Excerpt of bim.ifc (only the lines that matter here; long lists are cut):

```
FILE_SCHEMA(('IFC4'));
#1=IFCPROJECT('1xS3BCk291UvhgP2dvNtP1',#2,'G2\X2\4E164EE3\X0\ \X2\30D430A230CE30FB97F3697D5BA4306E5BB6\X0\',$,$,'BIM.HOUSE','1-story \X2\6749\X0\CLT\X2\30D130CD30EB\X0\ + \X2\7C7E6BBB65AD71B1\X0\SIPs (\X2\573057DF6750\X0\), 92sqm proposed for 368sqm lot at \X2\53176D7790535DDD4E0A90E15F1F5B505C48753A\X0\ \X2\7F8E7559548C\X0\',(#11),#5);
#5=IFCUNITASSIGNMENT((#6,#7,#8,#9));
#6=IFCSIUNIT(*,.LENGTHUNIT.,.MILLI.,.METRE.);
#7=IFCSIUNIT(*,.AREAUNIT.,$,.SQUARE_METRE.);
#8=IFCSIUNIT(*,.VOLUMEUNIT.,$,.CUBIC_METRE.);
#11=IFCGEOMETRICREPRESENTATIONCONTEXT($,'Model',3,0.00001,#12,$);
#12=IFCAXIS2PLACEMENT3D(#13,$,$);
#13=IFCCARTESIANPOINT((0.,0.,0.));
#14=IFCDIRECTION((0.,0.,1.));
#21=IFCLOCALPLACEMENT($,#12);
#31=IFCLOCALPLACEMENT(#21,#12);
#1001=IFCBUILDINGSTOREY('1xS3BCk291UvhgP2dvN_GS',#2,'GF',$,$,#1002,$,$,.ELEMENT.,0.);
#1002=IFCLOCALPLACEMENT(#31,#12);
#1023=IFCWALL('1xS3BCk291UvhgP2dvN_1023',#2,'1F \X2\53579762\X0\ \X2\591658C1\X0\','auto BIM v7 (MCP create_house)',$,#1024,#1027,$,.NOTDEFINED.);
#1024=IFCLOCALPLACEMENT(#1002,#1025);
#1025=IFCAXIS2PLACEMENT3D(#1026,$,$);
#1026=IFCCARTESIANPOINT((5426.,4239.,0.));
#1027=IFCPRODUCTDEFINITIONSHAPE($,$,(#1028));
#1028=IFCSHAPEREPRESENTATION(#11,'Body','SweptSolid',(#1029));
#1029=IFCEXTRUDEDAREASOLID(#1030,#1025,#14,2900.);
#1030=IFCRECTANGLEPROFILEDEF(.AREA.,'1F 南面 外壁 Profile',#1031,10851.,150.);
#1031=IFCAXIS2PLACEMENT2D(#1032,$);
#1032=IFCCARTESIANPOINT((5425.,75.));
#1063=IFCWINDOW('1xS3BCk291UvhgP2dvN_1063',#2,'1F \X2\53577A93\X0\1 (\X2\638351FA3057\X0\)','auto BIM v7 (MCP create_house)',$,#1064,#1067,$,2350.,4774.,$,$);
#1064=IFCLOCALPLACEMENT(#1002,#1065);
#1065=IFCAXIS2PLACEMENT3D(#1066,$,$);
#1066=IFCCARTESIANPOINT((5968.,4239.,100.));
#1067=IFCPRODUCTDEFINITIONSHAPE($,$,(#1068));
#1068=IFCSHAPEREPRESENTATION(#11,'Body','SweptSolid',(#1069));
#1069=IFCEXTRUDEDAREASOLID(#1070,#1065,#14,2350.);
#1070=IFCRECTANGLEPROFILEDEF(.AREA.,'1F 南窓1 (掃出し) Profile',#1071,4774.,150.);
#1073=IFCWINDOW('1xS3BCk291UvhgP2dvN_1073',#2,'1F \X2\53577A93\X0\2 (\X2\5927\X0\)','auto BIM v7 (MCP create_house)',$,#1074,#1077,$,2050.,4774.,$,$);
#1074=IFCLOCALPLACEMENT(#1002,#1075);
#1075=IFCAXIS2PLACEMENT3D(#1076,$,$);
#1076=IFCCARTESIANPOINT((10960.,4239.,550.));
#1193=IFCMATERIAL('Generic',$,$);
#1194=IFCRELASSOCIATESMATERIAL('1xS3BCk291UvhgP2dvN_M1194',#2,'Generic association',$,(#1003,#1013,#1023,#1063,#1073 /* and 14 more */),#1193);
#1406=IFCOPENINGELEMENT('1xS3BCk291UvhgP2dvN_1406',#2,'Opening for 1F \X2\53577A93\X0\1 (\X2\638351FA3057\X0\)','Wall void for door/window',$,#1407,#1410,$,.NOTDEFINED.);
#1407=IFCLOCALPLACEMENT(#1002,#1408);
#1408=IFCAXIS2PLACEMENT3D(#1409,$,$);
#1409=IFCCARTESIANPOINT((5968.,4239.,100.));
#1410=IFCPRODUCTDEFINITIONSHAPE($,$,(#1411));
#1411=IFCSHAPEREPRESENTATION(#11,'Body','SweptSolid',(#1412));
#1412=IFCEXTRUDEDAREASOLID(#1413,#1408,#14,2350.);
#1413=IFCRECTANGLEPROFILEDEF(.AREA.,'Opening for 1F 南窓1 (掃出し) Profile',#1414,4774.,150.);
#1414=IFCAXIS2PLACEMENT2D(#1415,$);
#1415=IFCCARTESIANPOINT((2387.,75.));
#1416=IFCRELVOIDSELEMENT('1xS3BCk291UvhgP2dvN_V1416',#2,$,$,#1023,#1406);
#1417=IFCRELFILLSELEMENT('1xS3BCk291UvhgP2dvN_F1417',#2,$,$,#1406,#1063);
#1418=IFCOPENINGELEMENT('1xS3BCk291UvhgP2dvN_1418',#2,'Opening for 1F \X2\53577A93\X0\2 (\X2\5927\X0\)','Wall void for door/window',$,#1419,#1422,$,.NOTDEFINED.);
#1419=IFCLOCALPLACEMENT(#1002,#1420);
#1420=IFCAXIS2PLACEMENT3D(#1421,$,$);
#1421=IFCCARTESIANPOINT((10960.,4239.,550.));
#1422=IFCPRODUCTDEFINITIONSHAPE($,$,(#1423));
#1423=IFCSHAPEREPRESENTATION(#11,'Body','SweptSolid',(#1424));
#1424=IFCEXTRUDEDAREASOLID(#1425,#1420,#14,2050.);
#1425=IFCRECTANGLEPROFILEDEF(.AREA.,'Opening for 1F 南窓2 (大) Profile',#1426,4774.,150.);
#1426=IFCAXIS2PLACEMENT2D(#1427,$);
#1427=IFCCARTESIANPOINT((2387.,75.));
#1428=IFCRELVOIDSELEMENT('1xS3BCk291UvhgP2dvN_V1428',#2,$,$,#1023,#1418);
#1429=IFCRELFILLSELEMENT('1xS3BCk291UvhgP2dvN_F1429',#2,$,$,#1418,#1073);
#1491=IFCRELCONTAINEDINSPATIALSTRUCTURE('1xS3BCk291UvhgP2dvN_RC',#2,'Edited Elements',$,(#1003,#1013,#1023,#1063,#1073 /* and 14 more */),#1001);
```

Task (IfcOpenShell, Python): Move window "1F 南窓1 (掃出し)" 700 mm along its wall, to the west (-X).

```python
import ifcopenshell
import ifcopenshell.api.geometry
import ifcopenshell.util.placement

model = ifcopenshell.open("bim.ifc")

window = model.by_guid("1xS3BCk291UvhgP2dvN_1063")
opening = window.FillsVoids[0].RelatingOpeningElement
wall = opening.VoidsElements[0].RelatingBuildingElement

wall_matrix = ifcopenshell.util.placement.get_local_placement(wall.ObjectPlacement)
shift = wall_matrix[:3, 0] * -700.0
before = ifcopenshell.util.placement.get_local_placement(window.ObjectPlacement)[:3, 3].copy()

# The window is not placed relative to its opening, so move both.
for product in (opening, window):
    matrix = ifcopenshell.util.placement.get_local_placement(product.ObjectPlacement)
    matrix[:3, 3] += shift
    ifcopenshell.api.geometry.edit_object_placement(model, product=product, matrix=matrix, is_si=False)

after = ifcopenshell.util.placement.get_local_placement(window.ObjectPlacement)[:3, 3]
print("window moved by", (after - before).round(3) + 0.0)

model.write("bim_updated.ifc")
```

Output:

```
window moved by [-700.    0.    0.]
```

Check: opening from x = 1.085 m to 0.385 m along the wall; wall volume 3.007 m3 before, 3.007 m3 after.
